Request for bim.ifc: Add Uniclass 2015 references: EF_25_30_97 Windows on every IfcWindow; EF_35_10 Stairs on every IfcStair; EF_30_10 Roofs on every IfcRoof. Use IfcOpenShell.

First a look at what the model holds.

```python
import ifcopenshell

model = ifcopenshell.open("bim.ifc")
print(model.schema)
print("classifications:", [c.Name for c in model.by_type("IfcClassification")])
for ifc_class in ("IfcDoor", "IfcRoof", "IfcStair", "IfcWall", "IfcWindow"):
    print(ifc_class, len(model.by_type(ifc_class)))
```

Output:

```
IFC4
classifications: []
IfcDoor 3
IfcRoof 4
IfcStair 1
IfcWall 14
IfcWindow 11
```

```python
import ifcopenshell
import ifcopenshell.api.classification

model = ifcopenshell.open("bim.ifc")

system = ifcopenshell.api.classification.add_classification(model, classification="Uniclass 2015")

codes = {
    "IfcWindow": ("EF_25_30_97", "Windows"),
    "IfcStair": ("EF_35_10", "Stairs"),
    "IfcRoof": ("EF_30_10", "Roofs"),
}
for ifc_class, (code, name) in codes.items():
    products = model.by_type(ifc_class)
    ifcopenshell.api.classification.add_reference(
        model, products=products, classification=system, identification=code, name=name
    )
    print(code, len(products))

model.write("bim_updated.ifc")
```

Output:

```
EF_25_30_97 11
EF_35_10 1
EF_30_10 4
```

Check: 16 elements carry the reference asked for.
